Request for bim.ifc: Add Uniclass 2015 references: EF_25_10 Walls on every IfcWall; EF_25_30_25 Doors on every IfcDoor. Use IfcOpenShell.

First a look at what the model holds.

```python
import ifcopenshell

model = ifcopenshell.open("bim.ifc")
print(model.schema)
print("classifications:", [c.Name for c in model.by_type("IfcClassification")])
for ifc_class in ("IfcDoor", "IfcRoof", "IfcStair", "IfcWall", "IfcWindow"):
    print(ifc_class, len(model.by_type(ifc_class)))
```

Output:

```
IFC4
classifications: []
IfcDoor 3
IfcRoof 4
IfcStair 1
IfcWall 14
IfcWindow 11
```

```python
import ifcopenshell
import ifcopenshell.api.classification

model = ifcopenshell.open("bim.ifc")

system = ifcopenshell.api.classification.add_classification(model, classification="Uniclass 2015")

codes = {
    "IfcWall": ("EF_25_10", "Walls"),
    "IfcDoor": ("EF_25_30_25", "Doors"),
}
for ifc_class, (code, name) in codes.items():
    products = model.by_type(ifc_class)
    ifcopenshell.api.classification.add_reference(
        model, products=products, classification=system, identification=code, name=name
    )
    print(code, len(products))

model.write("bim-out.ifc")
```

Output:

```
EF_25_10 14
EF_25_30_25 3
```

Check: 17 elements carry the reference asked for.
